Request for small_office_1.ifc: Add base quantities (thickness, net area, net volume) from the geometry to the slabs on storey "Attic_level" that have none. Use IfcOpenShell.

First a look at what the model holds.

```python
import ifcopenshell
import ifcopenshell.util.element
import ifcopenshell.util.unit

model = ifcopenshell.open("small_office_1.ifc")
print(model.schema)
for unit_type in ("LENGTHUNIT", "AREAUNIT", "VOLUMEUNIT"):
    print(unit_type, ifcopenshell.util.unit.calculate_unit_scale(model, unit_type))
storey = next(s for s in model.by_type("IfcBuildingStorey") if s.Name == "Attic_level")
slabs = [e for e in ifcopenshell.util.element.get_decomposition(storey) if e.is_a("IfcSlab")]
for e in sorted(slabs, key=lambda e: e.id()):
    print(e.id(), e.is_a(), e.Name, list(ifcopenshell.util.element.get_psets(e, qtos_only=True)), sep=" | ")
```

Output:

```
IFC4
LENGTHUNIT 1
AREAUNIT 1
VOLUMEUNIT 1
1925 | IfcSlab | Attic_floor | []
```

```python
import ifcopenshell
import ifcopenshell.api.pset
import ifcopenshell.geom
import ifcopenshell.util.element
import ifcopenshell.util.shape
import ifcopenshell.util.unit

model = ifcopenshell.open("small_office_1.ifc")
unit_scale = ifcopenshell.util.unit.calculate_unit_scale(model)
area_scale = ifcopenshell.util.unit.calculate_unit_scale(model, "AREAUNIT")
volume_scale = ifcopenshell.util.unit.calculate_unit_scale(model, "VOLUMEUNIT")
settings = ifcopenshell.geom.settings()

storey = next(s for s in model.by_type("IfcBuildingStorey") if s.Name == "Attic_level")
slabs = [e for e in ifcopenshell.util.element.get_decomposition(storey) if e.is_a("IfcSlab")]

for e in sorted(slabs, key=lambda e: e.id()):
    if ifcopenshell.util.element.get_psets(e, qtos_only=True, should_inherit=False):
        continue
    # Geometry comes back in metres, in the element's own axes.
    shape = ifcopenshell.geom.create_shape(settings, e)
    values = {
        "Width": ifcopenshell.util.shape.get_z(shape.geometry) / unit_scale,
        "NetArea": ifcopenshell.util.shape.get_footprint_area(shape.geometry) / area_scale,
        "NetVolume": ifcopenshell.util.shape.get_volume(shape.geometry) / volume_scale,
    }
    qto = ifcopenshell.api.pset.add_qto(model, product=e, name="Qto_SlabBaseQuantities")
    ifcopenshell.api.pset.edit_qto(model, qto=qto, properties=values)
    print(e.id(), {k: round(v, 3) for k, v in values.items()})

model.write("small_office_1_edited.ifc")
```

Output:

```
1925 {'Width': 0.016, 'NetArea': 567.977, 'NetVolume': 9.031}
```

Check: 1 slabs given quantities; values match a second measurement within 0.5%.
